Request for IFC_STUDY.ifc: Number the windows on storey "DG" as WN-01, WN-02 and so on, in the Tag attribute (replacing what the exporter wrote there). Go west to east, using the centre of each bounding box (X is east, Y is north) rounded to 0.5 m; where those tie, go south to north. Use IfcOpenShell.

First a look at what the model holds.

```python
import ifcopenshell
import ifcopenshell.util.element
import ifcopenshell.util.placement

model = ifcopenshell.open("IFC_STUDY.ifc")
print(model.schema)
storey = next(s for s in model.by_type("IfcBuildingStorey") if s.Name == "DG")
windows = [e for e in ifcopenshell.util.element.get_decomposition(storey) if e.is_a("IfcWindow")]
for e in sorted(windows, key=lambda e: e.id()):
    origin = ifcopenshell.util.placement.get_local_placement(e.ObjectPlacement)[:3, 3]
    print(e.id(), e.Tag, e.Name, origin.round(2) + 0.0, sep=" | ")
```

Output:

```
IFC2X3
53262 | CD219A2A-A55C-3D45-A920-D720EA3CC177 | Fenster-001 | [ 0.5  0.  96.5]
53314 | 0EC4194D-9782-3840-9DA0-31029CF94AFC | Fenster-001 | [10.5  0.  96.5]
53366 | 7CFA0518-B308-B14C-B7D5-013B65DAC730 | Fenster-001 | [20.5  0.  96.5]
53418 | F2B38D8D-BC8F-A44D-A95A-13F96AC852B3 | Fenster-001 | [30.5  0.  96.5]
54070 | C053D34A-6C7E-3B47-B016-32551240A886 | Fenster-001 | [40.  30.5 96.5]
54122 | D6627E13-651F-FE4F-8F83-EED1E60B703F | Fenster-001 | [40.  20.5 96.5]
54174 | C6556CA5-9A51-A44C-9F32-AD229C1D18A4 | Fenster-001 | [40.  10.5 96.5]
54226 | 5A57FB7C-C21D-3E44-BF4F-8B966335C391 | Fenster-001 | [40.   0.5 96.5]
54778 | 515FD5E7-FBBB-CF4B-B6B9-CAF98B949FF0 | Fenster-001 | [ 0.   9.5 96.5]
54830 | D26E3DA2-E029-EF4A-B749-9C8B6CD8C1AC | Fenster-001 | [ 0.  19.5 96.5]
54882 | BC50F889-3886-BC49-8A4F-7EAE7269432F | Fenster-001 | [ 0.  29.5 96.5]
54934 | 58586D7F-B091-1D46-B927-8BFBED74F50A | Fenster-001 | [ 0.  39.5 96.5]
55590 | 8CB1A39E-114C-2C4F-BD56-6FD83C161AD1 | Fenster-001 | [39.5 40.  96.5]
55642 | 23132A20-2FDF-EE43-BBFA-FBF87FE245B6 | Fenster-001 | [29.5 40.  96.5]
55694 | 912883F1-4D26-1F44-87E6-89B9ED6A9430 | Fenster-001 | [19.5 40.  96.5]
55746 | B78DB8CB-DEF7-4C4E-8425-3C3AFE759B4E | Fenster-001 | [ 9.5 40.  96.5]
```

```python
import ifcopenshell
import ifcopenshell.geom
import ifcopenshell.util.element
import ifcopenshell.util.shape

model = ifcopenshell.open("IFC_STUDY.ifc")
settings = ifcopenshell.geom.settings()
settings.set("use-world-coords", True)


def centre(element):
    shape = ifcopenshell.geom.create_shape(settings, element)
    return ifcopenshell.util.shape.get_bbox_centroid(shape.geometry)


storey = next(s for s in model.by_type("IfcBuildingStorey") if s.Name == "DG")
windows = [e for e in ifcopenshell.util.element.get_decomposition(storey) if e.is_a("IfcWindow")]

# Insertion points can sit at a corner or the storey origin, so sort by the geometry (in metres).
centres = {e: centre(e) for e in windows}
windows.sort(key=lambda e: (round(centres[e][0] / 0.5), centres[e][1]))

for i, e in enumerate(windows, start=1):
    number = f"WN-{i:02d}"
    e.Tag = number
    print(e.id(), number)

model.write("IFC_STUDY_v2.ifc")
```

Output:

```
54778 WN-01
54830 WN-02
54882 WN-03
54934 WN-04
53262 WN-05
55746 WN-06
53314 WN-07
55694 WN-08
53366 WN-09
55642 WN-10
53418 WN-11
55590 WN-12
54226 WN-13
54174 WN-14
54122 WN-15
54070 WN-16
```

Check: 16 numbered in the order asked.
